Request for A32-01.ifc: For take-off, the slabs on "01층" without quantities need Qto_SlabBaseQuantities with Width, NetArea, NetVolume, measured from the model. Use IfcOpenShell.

First a look at what the model holds.

```python
import ifcopenshell
import ifcopenshell.util.element
import ifcopenshell.util.unit

model = ifcopenshell.open("A32-01.ifc")
print(model.schema)
for unit_type in ("LENGTHUNIT", "AREAUNIT", "VOLUMEUNIT"):
    print(unit_type, ifcopenshell.util.unit.calculate_unit_scale(model, unit_type))
storey = next(s for s in model.by_type("IfcBuildingStorey") if s.Name == "01층")
slabs = [e for e in ifcopenshell.util.element.get_decomposition(storey) if e.is_a("IfcSlab")]
for e in sorted(slabs, key=lambda e: e.id()):
    print(e.id(), e.is_a(), e.Name, list(ifcopenshell.util.element.get_psets(e, qtos_only=True)), sep=" | ")
```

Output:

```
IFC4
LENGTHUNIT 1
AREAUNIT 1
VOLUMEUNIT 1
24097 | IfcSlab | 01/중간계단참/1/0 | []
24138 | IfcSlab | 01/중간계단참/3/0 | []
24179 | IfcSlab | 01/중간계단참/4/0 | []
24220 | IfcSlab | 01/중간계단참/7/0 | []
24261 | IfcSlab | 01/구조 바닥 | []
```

```python
import ifcopenshell
import ifcopenshell.api.pset
import ifcopenshell.geom
import ifcopenshell.util.element
import ifcopenshell.util.shape
import ifcopenshell.util.unit

model = ifcopenshell.open("A32-01.ifc")
unit_scale = ifcopenshell.util.unit.calculate_unit_scale(model)
area_scale = ifcopenshell.util.unit.calculate_unit_scale(model, "AREAUNIT")
volume_scale = ifcopenshell.util.unit.calculate_unit_scale(model, "VOLUMEUNIT")
settings = ifcopenshell.geom.settings()

storey = next(s for s in model.by_type("IfcBuildingStorey") if s.Name == "01층")
slabs = [e for e in ifcopenshell.util.element.get_decomposition(storey) if e.is_a("IfcSlab")]

for e in sorted(slabs, key=lambda e: e.id()):
    if ifcopenshell.util.element.get_psets(e, qtos_only=True, should_inherit=False):
        continue
    # Geometry comes back in metres, in the element's own axes.
    shape = ifcopenshell.geom.create_shape(settings, e)
    values = {
        "Width": ifcopenshell.util.shape.get_z(shape.geometry) / unit_scale,
        "NetArea": ifcopenshell.util.shape.get_footprint_area(shape.geometry) / area_scale,
        "NetVolume": ifcopenshell.util.shape.get_volume(shape.geometry) / volume_scale,
    }
    qto = ifcopenshell.api.pset.add_qto(model, product=e, name="Qto_SlabBaseQuantities")
    ifcopenshell.api.pset.edit_qto(model, qto=qto, properties=values)
    print(e.id(), {k: round(v, 3) for k, v in values.items()})

model.write("A32-01_updated.ifc")
```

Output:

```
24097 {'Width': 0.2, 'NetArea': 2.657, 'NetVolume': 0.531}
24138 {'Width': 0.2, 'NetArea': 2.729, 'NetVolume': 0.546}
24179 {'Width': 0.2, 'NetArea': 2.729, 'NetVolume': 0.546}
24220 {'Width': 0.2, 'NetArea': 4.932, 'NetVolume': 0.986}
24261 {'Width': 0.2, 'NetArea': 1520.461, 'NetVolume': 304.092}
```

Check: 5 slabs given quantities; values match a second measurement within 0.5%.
